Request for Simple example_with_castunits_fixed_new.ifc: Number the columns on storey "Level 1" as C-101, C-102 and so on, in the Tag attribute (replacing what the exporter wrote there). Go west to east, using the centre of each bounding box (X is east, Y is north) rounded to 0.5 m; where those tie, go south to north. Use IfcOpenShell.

First a look at what the model holds.

```python
import ifcopenshell
import ifcopenshell.util.element
import ifcopenshell.util.placement

model = ifcopenshell.open("Simple example_with_castunits_fixed_new.ifc")
print(model.schema)
storey = next(s for s in model.by_type("IfcBuildingStorey") if s.Name == "Level 1")
columns = [e for e in ifcopenshell.util.element.get_decomposition(storey) if e.is_a("IfcColumn")]
for e in sorted(columns, key=lambda e: e.id()):
    origin = ifcopenshell.util.placement.get_local_placement(e.ObjectPlacement)[:3, 3]
    print(e.id(), e.Tag, e.Name, origin.round(2) + 0.0, sep=" | ")
```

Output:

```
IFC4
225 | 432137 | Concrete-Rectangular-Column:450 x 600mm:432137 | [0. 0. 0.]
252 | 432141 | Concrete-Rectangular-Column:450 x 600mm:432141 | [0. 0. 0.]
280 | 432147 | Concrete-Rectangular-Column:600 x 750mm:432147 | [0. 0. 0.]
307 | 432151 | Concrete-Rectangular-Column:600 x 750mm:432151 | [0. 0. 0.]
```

```python
import ifcopenshell
import ifcopenshell.geom
import ifcopenshell.util.element
import ifcopenshell.util.shape

model = ifcopenshell.open("Simple example_with_castunits_fixed_new.ifc")
settings = ifcopenshell.geom.settings()
settings.set("use-world-coords", True)


def centre(element):
    shape = ifcopenshell.geom.create_shape(settings, element)
    return ifcopenshell.util.shape.get_bbox_centroid(shape.geometry)


storey = next(s for s in model.by_type("IfcBuildingStorey") if s.Name == "Level 1")
columns = [e for e in ifcopenshell.util.element.get_decomposition(storey) if e.is_a("IfcColumn")]

# Insertion points can sit at a corner or the storey origin, so sort by the geometry (in metres).
centres = {e: centre(e) for e in columns}
columns.sort(key=lambda e: (round(centres[e][0] / 0.5), centres[e][1]))

for i, e in enumerate(columns, start=1):
    number = f"C-1{i:02d}"
    e.Tag = number
    print(e.id(), number)

model.write("Simple example_with_castunits_fixed_new_rev.ifc")
```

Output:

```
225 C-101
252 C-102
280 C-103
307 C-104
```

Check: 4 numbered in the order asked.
